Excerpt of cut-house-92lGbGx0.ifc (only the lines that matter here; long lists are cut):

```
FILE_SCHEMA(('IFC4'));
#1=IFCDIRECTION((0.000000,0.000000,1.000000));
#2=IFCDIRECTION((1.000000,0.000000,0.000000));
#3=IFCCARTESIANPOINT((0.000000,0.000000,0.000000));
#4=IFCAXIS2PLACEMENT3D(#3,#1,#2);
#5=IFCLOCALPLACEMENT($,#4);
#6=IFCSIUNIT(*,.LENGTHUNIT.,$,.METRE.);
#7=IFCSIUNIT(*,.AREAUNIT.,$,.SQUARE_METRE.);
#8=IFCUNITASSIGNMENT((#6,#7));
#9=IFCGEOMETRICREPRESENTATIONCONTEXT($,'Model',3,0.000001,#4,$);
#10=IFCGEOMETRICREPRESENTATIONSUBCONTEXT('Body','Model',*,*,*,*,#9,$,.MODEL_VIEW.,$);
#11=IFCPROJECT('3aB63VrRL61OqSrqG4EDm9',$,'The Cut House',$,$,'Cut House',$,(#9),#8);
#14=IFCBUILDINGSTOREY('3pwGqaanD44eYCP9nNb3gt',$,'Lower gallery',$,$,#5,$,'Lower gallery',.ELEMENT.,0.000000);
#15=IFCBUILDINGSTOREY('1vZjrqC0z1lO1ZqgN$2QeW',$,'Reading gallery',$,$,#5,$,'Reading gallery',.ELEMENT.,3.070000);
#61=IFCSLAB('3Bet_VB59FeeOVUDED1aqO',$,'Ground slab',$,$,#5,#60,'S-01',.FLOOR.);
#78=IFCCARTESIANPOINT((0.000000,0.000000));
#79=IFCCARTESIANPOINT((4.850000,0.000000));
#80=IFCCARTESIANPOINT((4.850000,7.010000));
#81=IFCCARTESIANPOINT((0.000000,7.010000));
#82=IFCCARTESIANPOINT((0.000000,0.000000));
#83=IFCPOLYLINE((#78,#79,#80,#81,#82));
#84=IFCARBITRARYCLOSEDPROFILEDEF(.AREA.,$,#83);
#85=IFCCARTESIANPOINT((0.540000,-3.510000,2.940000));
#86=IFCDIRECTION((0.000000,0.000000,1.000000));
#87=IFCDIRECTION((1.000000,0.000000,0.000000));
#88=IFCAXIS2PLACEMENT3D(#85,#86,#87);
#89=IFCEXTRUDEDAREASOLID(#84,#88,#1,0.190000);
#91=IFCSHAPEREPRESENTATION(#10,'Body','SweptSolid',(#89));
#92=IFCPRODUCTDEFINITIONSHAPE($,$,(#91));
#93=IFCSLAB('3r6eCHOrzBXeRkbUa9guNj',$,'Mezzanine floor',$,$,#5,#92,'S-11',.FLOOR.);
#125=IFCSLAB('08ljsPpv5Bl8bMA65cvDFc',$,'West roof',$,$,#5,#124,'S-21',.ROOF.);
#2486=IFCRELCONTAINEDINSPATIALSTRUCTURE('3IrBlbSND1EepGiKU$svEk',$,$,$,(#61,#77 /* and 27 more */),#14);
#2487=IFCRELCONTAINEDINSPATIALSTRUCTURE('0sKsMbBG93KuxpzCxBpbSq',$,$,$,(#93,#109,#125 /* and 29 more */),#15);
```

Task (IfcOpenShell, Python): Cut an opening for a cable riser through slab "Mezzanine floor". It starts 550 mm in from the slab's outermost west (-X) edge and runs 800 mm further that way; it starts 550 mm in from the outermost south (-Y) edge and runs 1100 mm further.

```python
import numpy as np
import ifcopenshell
import ifcopenshell.api.feature
import ifcopenshell.api.geometry
import ifcopenshell.api.root
import ifcopenshell.geom
import ifcopenshell.util.placement
import ifcopenshell.util.representation
import ifcopenshell.util.shape
import ifcopenshell.util.unit

model = ifcopenshell.open("cut-house-92lGbGx0.ifc")
unit_scale = ifcopenshell.util.unit.calculate_unit_scale(model)
settings = ifcopenshell.geom.settings()


def volume(element):
    """Net volume in cubic metres, openings subtracted."""
    shape = ifcopenshell.geom.create_shape(settings, element)
    return ifcopenshell.util.shape.get_volume(shape.geometry)


slab = model.by_guid("3r6eCHOrzBXeRkbUa9guNj")
before = volume(slab)

# Extent in the slab's own axes, in metres. The edges named are its -X and -Y sides.
slab_shape = ifcopenshell.geom.create_shape(settings, slab)
vertices = ifcopenshell.util.shape.get_vertices(slab_shape.geometry)
x_min, y_min, bottom = vertices.min(axis=0)
top = vertices[:, 2].max()

opening = ifcopenshell.api.root.create_entity(model, ifc_class="IfcOpeningElement", name="Cable riser opening", predefined_type="OPENING")
context = ifcopenshell.util.representation.get_context(model, "Model", "Body", "MODEL_VIEW")
width, depth = 0.8, 1.1
outline = [(0.0, 0.0), (width, 0.0), (width, depth), (0.0, depth), (0.0, 0.0)]
# Overshoot both faces by 50 mm so the cut is clean.
shape = ifcopenshell.api.geometry.add_slab_representation(
    model, context=context, depth=top - bottom + 0.1, polyline=outline
)
ifcopenshell.api.geometry.assign_representation(model, product=opening, representation=shape)

matrix = ifcopenshell.util.placement.get_local_placement(slab.ObjectPlacement)
matrix[:, 3] = matrix @ np.append(np.array([x_min + 0.55, y_min + 0.55, bottom - 0.05]) / unit_scale, 1.0)
ifcopenshell.api.geometry.edit_object_placement(model, product=opening, matrix=matrix, is_si=False)
ifcopenshell.api.feature.add_feature(model, feature=opening, element=slab)

after = volume(slab)

print(f"slab volume {before:.3f} -> {after:.3f} m3")

model.write("cut-house-92lGbGx0_rev.ifc")
```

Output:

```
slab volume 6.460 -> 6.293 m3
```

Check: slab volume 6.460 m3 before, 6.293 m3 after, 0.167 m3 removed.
